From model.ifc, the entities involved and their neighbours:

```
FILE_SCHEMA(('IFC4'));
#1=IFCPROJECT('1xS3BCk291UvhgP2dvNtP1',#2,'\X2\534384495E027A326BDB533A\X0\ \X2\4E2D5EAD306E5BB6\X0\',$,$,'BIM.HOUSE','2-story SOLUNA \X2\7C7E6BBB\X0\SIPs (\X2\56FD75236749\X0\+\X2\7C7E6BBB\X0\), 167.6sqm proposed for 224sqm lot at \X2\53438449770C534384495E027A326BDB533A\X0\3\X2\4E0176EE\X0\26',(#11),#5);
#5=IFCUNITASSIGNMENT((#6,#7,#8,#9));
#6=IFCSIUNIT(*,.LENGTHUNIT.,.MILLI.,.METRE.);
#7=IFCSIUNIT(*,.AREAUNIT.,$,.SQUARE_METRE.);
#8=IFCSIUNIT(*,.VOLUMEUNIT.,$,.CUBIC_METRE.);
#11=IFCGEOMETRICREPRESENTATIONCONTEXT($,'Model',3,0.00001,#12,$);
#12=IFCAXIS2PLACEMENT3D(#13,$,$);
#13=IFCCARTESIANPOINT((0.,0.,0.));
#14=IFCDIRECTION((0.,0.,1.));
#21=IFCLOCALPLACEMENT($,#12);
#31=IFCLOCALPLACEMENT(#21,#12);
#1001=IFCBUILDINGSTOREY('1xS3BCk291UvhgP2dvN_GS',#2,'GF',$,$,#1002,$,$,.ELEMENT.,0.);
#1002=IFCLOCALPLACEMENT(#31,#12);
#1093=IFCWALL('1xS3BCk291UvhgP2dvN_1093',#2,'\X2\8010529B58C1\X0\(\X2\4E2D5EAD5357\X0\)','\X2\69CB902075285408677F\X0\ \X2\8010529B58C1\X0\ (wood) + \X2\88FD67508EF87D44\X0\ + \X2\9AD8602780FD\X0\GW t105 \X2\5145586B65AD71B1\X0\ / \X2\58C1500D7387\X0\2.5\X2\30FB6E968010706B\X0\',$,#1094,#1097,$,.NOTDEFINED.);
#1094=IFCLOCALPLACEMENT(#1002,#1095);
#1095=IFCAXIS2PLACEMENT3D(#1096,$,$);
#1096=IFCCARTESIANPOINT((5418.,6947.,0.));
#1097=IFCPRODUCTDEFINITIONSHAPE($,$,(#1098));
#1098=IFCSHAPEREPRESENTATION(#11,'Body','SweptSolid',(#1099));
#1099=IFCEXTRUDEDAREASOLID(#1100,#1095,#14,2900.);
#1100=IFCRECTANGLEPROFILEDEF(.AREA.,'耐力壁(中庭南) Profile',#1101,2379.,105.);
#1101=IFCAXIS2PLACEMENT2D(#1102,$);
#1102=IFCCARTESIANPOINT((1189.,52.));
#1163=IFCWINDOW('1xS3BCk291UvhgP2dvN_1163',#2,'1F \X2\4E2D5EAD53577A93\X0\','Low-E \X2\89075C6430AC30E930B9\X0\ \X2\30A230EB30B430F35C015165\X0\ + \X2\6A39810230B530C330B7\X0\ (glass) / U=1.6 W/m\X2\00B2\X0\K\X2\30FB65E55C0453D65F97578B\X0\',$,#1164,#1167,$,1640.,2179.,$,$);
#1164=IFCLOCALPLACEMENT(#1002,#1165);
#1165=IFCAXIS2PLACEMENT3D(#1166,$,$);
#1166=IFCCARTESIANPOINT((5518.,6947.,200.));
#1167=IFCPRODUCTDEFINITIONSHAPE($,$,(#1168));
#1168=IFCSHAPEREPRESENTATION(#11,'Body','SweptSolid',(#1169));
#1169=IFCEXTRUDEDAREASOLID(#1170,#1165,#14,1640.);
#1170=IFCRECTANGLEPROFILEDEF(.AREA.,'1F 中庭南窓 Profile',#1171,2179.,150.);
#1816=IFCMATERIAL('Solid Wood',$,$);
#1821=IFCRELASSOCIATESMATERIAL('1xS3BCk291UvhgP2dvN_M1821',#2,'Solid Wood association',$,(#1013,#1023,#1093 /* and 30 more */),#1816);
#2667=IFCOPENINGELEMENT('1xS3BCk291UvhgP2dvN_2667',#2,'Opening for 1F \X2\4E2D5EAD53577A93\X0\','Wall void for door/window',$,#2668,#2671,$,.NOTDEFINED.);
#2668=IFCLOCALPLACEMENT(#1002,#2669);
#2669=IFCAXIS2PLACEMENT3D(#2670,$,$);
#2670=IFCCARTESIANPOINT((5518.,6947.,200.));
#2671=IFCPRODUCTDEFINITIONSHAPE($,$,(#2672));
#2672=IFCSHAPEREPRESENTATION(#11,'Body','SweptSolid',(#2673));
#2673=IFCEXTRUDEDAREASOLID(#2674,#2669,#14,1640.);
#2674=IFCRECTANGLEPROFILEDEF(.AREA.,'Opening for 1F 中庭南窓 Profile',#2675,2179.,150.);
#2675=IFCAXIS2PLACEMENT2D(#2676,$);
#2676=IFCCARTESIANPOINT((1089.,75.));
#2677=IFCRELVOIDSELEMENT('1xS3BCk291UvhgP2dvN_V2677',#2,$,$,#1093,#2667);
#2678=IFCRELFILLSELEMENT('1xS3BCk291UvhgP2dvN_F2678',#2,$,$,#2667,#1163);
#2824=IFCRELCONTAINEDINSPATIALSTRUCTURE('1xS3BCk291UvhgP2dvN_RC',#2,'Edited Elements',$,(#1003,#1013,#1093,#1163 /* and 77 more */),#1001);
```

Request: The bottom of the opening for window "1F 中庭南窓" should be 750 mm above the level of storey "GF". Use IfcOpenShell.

```python
import numpy as np
import ifcopenshell
import ifcopenshell.api.geometry
import ifcopenshell.geom
import ifcopenshell.util.element
import ifcopenshell.util.placement
import ifcopenshell.util.shape
import ifcopenshell.util.unit

model = ifcopenshell.open("model.ifc")
unit_scale = ifcopenshell.util.unit.calculate_unit_scale(model)

window = model.by_guid("1xS3BCk291UvhgP2dvN_1163")
opening = window.FillsVoids[0].RelatingOpeningElement
storey = ifcopenshell.util.element.get_container(window, ifc_class="IfcBuildingStorey")
level = ifcopenshell.util.placement.get_local_placement(storey.ObjectPlacement)[2, 3]

# The opening's origin need not be at the sill, so measure its lowest point.
shape = ifcopenshell.geom.create_shape(ifcopenshell.geom.settings(), opening)
bottom = ifcopenshell.util.shape.get_shape_bottom_elevation(shape, shape.geometry) / unit_scale
dz = level + 0.75 / unit_scale - bottom

shift = np.array([0.0, 0.0, dz])
# The window is not placed relative to its opening, so move both.
for product in (opening, window):
    matrix = ifcopenshell.util.placement.get_local_placement(product.ObjectPlacement)
    matrix[:3, 3] += shift
    ifcopenshell.api.geometry.edit_object_placement(model, product=product, matrix=matrix, is_si=False)

print(f"moved by {dz * unit_scale:+.3f} m")

model.write("model_edited.ifc")
```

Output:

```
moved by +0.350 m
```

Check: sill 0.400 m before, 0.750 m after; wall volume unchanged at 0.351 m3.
